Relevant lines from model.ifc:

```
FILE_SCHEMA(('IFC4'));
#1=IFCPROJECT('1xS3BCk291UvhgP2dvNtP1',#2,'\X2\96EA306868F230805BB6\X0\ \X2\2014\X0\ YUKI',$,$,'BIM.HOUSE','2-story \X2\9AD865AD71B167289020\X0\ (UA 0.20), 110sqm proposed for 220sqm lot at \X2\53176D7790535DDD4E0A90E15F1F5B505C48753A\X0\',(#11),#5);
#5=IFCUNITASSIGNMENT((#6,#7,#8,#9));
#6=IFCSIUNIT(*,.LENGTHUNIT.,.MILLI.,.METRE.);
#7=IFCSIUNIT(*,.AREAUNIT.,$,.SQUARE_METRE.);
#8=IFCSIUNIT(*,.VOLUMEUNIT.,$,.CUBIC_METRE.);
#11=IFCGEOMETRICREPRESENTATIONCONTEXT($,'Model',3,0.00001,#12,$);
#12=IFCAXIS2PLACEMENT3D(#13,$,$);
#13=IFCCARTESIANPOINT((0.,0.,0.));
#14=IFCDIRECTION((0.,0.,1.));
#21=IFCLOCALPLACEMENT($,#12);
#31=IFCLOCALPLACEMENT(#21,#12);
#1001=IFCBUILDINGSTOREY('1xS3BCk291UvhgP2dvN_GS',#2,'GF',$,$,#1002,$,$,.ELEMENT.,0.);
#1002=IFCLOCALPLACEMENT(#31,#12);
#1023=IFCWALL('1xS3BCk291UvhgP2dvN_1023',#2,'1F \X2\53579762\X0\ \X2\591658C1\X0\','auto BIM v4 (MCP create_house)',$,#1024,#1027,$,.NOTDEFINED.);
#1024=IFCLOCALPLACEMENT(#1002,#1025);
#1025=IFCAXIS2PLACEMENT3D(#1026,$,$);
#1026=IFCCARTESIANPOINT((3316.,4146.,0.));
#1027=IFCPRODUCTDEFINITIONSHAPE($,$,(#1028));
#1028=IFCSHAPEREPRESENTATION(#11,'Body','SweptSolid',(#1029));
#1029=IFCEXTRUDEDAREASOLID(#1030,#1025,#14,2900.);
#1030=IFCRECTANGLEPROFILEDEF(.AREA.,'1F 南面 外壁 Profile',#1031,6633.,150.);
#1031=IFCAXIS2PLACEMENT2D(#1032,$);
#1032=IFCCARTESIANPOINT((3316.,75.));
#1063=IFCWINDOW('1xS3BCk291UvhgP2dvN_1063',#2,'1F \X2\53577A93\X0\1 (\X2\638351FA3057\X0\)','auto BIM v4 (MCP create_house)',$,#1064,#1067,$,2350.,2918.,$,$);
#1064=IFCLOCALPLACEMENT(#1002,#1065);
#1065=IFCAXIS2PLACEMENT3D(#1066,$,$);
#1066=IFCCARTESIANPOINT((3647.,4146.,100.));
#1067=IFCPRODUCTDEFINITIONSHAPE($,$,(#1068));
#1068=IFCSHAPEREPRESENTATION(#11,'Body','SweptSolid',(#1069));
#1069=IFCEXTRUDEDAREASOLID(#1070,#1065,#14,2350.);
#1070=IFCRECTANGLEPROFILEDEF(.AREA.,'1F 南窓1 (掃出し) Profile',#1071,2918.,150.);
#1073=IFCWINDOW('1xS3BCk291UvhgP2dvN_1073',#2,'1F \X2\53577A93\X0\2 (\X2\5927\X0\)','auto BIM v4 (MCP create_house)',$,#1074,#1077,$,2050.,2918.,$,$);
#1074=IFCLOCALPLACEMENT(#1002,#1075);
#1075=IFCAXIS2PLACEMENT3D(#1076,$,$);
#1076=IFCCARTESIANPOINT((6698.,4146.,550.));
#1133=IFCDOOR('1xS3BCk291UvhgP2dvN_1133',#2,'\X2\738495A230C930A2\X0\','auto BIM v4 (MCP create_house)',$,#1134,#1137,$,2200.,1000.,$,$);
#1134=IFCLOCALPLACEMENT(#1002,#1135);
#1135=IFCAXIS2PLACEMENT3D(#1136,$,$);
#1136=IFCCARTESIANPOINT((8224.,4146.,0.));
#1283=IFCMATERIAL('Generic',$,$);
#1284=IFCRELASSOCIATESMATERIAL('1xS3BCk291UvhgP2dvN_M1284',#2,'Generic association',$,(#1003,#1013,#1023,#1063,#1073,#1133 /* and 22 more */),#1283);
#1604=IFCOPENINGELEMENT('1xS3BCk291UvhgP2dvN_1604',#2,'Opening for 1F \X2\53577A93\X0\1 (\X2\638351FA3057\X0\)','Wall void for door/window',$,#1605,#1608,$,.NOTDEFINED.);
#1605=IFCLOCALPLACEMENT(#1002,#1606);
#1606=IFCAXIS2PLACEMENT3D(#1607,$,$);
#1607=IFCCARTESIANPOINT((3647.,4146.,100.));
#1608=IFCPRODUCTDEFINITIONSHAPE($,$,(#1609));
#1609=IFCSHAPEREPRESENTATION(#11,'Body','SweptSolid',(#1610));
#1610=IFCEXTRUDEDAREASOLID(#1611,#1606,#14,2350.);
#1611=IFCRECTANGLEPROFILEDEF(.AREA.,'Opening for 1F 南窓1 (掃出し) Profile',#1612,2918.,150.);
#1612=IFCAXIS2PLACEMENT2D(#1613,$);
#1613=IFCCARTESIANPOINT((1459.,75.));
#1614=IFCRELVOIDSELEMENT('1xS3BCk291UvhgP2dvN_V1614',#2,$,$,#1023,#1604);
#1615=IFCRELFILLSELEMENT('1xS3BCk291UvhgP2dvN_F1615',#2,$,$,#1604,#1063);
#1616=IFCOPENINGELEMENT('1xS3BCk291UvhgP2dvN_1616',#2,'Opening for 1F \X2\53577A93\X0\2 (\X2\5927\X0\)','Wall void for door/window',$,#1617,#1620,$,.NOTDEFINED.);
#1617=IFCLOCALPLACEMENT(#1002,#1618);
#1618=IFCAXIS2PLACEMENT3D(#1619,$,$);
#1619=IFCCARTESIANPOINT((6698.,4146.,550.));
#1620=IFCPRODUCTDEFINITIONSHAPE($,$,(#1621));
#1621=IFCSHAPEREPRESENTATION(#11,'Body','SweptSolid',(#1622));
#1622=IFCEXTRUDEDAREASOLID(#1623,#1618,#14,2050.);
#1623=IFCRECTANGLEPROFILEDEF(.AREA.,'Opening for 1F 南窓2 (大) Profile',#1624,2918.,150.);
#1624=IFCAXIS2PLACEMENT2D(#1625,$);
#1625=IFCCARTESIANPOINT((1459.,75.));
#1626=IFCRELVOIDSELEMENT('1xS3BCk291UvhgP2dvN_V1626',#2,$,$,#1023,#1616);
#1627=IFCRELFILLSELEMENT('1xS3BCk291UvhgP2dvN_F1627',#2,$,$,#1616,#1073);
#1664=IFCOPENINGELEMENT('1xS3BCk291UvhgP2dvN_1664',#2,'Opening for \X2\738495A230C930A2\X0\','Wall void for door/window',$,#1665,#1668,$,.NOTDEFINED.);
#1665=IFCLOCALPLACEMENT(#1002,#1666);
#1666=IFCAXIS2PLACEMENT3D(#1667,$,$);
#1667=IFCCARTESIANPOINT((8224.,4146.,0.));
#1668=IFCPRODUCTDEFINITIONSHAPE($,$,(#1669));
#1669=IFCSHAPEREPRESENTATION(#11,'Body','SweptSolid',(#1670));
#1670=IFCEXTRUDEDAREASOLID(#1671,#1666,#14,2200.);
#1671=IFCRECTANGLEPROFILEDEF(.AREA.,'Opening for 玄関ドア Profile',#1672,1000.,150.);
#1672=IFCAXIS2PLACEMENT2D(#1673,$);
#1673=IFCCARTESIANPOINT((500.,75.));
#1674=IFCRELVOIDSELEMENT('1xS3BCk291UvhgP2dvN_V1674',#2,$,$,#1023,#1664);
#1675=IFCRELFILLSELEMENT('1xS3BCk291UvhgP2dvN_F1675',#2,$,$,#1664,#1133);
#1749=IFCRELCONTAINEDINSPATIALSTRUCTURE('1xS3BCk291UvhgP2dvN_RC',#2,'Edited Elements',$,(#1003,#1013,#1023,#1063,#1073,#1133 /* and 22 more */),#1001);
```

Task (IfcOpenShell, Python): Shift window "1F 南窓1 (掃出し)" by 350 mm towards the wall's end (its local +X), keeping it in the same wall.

```python
import ifcopenshell
import ifcopenshell.api.geometry
import ifcopenshell.util.placement
import ifcopenshell.util.unit

model = ifcopenshell.open("model.ifc")
unit_scale = ifcopenshell.util.unit.calculate_unit_scale(model)

window = model.by_guid("1xS3BCk291UvhgP2dvN_1063")
opening = window.FillsVoids[0].RelatingOpeningElement
wall = opening.VoidsElements[0].RelatingBuildingElement

wall_matrix = ifcopenshell.util.placement.get_local_placement(wall.ObjectPlacement)
shift = wall_matrix[:3, 0] * 0.35 / unit_scale
before = ifcopenshell.util.placement.get_local_placement(window.ObjectPlacement)[:3, 3].copy()

# The window is not placed relative to its opening, so move both.
for product in (opening, window):
    matrix = ifcopenshell.util.placement.get_local_placement(product.ObjectPlacement)
    matrix[:3, 3] += shift
    ifcopenshell.api.geometry.edit_object_placement(model, product=product, matrix=matrix, is_si=False)

after = ifcopenshell.util.placement.get_local_placement(window.ObjectPlacement)[:3, 3]
print("window moved by", (after - before).round(3) + 0.0)

model.write("model_edited.ifc")
```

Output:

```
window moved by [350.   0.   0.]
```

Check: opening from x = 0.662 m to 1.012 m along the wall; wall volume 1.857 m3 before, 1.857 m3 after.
